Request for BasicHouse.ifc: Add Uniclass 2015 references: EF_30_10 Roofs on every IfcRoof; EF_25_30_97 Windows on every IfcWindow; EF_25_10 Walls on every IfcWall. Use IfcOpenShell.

First a look at what the model holds.

```python
import ifcopenshell

model = ifcopenshell.open("BasicHouse.ifc")
print(model.schema)
print("classifications:", [c.Name for c in model.by_type("IfcClassification")])
for ifc_class in ("IfcDoor", "IfcRoof", "IfcStair", "IfcWall", "IfcWindow"):
    print(ifc_class, len(model.by_type(ifc_class)))
```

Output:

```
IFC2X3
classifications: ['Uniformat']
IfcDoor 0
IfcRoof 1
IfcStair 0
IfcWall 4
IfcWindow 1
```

```python
import ifcopenshell
import ifcopenshell.api.classification

model = ifcopenshell.open("BasicHouse.ifc")

# IFC2X3 requires Source and Edition and has no link from the project to the system.
system = model.create_entity("IfcClassification", Source="NBS", Edition="2015", Name="Uniclass 2015")

codes = {
    "IfcRoof": ("EF_30_10", "Roofs"),
    "IfcWindow": ("EF_25_30_97", "Windows"),
    "IfcWall": ("EF_25_10", "Walls"),
}
for ifc_class, (code, name) in codes.items():
    products = model.by_type(ifc_class)
    ifcopenshell.api.classification.add_reference(
        model, products=products, classification=system, identification=code, name=name
    )
    print(code, len(products))

model.write("BasicHouse_rev.ifc")
```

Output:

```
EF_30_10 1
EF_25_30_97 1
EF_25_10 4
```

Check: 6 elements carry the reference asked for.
